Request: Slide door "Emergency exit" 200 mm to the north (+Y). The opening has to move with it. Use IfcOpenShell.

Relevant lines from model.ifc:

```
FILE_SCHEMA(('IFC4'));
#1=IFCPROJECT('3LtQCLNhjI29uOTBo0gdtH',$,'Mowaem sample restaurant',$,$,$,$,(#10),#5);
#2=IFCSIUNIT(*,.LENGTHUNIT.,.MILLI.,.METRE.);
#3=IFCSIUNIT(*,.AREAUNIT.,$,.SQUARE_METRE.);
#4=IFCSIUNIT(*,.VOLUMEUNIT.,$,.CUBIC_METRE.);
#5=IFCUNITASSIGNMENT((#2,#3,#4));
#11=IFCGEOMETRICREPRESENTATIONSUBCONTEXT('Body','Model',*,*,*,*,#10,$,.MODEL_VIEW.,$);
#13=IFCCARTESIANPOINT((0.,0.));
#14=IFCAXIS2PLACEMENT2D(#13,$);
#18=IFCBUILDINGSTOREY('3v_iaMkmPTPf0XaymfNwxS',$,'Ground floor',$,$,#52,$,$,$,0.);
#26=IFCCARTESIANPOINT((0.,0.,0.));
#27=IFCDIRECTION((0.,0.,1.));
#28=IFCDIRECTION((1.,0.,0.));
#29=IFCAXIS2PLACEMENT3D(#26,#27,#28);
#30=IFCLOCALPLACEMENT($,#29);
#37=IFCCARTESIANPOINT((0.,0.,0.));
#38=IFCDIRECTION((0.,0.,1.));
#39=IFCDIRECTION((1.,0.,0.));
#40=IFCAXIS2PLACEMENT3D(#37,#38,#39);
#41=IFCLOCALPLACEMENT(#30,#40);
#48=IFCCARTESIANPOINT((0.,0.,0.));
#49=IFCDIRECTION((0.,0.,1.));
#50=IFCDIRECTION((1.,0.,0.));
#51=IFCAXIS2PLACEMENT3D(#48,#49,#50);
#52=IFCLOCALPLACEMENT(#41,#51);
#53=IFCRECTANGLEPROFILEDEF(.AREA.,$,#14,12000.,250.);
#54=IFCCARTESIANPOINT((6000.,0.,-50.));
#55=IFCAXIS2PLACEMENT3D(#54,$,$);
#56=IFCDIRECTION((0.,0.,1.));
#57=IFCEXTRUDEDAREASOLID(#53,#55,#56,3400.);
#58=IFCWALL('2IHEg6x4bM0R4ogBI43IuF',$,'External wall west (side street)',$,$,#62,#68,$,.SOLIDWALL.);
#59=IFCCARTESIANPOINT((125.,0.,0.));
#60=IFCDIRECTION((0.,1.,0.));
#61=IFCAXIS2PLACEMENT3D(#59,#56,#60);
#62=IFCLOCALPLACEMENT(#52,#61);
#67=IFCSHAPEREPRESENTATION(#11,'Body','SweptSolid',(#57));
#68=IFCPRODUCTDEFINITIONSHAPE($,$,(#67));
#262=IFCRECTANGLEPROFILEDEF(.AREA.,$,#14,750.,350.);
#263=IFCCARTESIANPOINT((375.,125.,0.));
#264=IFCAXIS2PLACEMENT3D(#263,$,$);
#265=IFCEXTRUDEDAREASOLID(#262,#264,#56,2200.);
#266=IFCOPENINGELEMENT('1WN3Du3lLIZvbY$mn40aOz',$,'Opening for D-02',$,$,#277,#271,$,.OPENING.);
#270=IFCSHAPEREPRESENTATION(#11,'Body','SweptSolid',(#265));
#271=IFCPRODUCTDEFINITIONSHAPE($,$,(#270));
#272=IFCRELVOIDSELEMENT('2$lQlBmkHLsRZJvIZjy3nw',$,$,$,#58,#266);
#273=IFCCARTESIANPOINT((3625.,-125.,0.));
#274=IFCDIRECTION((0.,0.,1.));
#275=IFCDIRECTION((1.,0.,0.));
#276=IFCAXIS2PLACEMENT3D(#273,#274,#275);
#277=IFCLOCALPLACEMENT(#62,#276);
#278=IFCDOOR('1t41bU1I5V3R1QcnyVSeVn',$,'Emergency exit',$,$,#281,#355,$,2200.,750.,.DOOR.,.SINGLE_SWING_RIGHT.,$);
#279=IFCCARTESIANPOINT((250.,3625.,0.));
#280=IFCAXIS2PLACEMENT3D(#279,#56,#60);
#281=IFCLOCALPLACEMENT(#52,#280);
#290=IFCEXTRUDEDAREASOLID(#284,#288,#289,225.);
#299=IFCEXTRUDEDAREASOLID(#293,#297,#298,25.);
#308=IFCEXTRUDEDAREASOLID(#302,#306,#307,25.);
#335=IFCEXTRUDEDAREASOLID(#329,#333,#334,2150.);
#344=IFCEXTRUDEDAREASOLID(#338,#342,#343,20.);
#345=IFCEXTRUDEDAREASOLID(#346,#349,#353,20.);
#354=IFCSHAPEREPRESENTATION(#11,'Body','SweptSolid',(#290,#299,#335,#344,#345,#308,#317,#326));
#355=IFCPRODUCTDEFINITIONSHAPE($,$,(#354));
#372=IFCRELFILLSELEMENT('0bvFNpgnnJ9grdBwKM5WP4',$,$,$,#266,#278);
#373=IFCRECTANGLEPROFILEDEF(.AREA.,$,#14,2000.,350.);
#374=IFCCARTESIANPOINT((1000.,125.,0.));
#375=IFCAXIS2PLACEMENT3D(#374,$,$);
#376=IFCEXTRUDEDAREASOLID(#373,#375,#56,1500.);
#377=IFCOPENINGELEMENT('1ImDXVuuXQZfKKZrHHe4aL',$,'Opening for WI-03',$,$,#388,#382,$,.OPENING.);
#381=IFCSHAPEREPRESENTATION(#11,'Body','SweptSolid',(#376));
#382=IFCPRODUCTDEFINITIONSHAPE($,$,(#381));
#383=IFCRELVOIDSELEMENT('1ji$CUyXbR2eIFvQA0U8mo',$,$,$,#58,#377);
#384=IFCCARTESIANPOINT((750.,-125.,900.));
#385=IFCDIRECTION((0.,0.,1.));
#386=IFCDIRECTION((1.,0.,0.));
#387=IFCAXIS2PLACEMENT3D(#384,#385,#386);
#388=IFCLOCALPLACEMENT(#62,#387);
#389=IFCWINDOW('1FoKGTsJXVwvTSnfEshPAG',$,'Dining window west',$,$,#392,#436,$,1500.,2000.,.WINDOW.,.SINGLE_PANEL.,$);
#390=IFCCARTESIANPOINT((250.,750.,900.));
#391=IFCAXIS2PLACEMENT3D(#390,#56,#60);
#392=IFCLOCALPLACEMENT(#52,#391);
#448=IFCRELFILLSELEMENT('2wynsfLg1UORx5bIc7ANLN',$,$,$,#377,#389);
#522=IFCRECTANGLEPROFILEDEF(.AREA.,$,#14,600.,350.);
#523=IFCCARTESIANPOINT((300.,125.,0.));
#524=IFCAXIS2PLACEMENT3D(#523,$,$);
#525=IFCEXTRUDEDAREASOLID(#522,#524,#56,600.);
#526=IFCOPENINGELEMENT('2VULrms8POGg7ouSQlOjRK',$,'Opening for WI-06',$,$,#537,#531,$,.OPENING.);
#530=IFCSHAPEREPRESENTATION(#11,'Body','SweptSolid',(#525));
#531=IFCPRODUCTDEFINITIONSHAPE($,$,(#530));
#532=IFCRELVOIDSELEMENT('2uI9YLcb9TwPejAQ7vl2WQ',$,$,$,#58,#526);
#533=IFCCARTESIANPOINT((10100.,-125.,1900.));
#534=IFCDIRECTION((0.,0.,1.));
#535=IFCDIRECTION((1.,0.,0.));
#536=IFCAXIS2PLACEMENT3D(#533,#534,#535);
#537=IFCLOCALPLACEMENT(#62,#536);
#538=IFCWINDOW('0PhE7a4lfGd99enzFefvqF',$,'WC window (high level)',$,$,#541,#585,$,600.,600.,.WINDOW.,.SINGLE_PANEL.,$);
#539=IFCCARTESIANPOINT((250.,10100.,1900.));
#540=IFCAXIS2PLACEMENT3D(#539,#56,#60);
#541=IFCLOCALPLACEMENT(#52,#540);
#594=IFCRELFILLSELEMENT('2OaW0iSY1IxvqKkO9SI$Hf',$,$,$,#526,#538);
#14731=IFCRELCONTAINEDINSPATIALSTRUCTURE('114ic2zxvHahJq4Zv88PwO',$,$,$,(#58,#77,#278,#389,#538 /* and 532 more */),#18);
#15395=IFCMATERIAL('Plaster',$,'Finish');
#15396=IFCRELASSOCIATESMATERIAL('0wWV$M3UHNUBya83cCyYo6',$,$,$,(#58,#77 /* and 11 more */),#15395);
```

```python
import ifcopenshell
import ifcopenshell.api.geometry
import ifcopenshell.util.placement
import ifcopenshell.util.unit

model = ifcopenshell.open("model.ifc")
unit_scale = ifcopenshell.util.unit.calculate_unit_scale(model)

door = model.by_guid("1t41bU1I5V3R1QcnyVSeVn")
opening = door.FillsVoids[0].RelatingOpeningElement
wall = opening.VoidsElements[0].RelatingBuildingElement

wall_matrix = ifcopenshell.util.placement.get_local_placement(wall.ObjectPlacement)
shift = wall_matrix[:3, 0] * 0.2 / unit_scale
before = ifcopenshell.util.placement.get_local_placement(door.ObjectPlacement)[:3, 3].copy()

# The door is not placed relative to its opening, so move both.
for product in (opening, door):
    matrix = ifcopenshell.util.placement.get_local_placement(product.ObjectPlacement)
    matrix[:3, 3] += shift
    ifcopenshell.api.geometry.edit_object_placement(model, product=product, matrix=matrix, is_si=False)

after = ifcopenshell.util.placement.get_local_placement(door.ObjectPlacement)[:3, 3]
print("door moved by", (after - before).round(3) + 0.0)

model.write("model-out.ifc")
```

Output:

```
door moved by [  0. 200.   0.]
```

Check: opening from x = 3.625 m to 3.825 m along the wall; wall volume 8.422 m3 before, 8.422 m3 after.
